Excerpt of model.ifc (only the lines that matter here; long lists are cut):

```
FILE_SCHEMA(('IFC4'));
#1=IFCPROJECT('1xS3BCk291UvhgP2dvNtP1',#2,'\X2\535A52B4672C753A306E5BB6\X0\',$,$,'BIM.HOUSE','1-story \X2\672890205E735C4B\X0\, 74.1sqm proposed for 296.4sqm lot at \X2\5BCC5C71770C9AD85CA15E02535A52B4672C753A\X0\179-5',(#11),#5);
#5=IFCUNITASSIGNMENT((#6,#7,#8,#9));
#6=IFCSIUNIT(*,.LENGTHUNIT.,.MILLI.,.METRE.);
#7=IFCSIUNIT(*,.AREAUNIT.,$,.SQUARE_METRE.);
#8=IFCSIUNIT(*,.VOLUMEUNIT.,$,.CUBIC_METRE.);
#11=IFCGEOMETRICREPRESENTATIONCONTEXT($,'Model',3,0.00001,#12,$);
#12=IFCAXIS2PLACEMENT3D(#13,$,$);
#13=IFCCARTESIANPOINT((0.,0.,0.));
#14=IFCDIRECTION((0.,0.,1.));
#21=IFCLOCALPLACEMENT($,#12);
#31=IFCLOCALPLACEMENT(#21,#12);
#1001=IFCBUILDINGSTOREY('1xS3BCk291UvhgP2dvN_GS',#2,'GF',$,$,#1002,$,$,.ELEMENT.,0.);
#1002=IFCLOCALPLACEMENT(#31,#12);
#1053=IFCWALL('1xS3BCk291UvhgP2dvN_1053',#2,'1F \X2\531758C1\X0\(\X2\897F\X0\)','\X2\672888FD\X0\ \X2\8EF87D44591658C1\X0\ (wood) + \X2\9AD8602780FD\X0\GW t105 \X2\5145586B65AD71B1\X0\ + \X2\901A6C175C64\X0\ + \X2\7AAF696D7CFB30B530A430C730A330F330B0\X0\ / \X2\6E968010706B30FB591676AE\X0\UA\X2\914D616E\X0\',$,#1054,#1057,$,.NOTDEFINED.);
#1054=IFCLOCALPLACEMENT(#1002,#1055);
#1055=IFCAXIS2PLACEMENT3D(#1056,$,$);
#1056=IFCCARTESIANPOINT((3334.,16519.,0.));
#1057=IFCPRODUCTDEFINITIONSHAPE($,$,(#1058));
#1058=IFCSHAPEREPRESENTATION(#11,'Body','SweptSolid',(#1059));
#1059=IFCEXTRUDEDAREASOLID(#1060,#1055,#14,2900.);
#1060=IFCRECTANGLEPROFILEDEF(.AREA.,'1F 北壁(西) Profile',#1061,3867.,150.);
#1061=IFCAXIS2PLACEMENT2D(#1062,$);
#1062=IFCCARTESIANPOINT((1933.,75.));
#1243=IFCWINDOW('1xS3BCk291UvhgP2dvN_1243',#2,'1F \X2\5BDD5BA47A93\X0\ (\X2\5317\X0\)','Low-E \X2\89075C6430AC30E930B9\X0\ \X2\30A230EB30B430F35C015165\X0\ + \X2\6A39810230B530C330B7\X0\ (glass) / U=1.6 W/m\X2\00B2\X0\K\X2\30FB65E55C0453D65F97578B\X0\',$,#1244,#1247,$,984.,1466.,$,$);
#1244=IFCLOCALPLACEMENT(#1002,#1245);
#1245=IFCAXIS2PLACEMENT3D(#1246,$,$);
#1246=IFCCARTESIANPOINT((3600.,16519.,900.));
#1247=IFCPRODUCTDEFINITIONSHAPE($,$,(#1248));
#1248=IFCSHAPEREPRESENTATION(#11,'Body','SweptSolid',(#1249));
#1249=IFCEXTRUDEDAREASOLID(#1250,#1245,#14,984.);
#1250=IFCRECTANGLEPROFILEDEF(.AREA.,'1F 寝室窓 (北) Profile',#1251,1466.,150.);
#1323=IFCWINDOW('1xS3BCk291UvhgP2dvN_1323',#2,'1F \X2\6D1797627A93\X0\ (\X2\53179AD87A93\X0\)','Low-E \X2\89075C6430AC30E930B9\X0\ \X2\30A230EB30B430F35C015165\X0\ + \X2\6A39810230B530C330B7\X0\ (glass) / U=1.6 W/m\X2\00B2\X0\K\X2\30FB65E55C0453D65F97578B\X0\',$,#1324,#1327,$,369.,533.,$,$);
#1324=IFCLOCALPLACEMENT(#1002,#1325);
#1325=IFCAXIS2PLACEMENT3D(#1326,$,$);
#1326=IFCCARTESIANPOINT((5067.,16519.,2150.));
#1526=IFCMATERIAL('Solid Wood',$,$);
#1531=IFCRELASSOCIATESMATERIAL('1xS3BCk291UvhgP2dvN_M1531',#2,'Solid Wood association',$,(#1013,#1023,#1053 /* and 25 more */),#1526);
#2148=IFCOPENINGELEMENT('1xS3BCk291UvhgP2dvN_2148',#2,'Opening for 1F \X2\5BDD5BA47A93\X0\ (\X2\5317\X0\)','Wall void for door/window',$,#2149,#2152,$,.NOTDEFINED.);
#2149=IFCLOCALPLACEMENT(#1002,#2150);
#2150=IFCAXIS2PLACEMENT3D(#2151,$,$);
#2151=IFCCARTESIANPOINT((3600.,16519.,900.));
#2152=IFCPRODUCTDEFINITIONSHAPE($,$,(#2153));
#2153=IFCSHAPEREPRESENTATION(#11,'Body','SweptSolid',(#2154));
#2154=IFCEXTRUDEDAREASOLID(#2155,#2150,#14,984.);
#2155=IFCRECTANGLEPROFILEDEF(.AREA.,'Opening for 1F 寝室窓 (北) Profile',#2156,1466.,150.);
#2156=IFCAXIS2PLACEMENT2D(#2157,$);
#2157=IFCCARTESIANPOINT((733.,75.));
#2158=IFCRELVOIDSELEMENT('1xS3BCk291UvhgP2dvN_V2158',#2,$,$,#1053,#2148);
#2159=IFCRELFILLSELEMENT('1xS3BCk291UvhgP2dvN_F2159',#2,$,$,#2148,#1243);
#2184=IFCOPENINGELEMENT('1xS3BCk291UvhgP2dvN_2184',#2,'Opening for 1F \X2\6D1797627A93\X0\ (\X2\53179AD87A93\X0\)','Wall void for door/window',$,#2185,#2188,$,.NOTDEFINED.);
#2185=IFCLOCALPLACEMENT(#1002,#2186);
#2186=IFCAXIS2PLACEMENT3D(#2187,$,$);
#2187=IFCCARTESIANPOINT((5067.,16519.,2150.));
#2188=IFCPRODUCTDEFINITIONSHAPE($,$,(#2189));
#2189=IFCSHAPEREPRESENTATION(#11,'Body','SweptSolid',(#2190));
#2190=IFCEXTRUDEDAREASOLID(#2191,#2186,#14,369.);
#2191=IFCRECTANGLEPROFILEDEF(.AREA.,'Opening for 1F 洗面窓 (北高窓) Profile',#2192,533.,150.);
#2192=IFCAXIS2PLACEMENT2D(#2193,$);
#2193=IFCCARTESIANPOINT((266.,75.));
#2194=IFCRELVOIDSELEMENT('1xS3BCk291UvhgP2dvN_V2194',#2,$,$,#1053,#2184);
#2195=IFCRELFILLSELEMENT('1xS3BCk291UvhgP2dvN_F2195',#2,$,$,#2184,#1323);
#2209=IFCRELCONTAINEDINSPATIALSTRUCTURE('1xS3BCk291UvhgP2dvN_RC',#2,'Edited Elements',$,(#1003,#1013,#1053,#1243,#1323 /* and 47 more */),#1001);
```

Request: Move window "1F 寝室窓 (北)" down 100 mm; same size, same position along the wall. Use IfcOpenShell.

```python
import numpy as np
import ifcopenshell
import ifcopenshell.api.geometry
import ifcopenshell.util.placement
import ifcopenshell.util.unit

model = ifcopenshell.open("model.ifc")
unit_scale = ifcopenshell.util.unit.calculate_unit_scale(model)

window = model.by_guid("1xS3BCk291UvhgP2dvN_1243")
opening = window.FillsVoids[0].RelatingOpeningElement
dz = -0.1 / unit_scale

shift = np.array([0.0, 0.0, dz])
# The window is not placed relative to its opening, so move both.
for product in (opening, window):
    matrix = ifcopenshell.util.placement.get_local_placement(product.ObjectPlacement)
    matrix[:3, 3] += shift
    ifcopenshell.api.geometry.edit_object_placement(model, product=product, matrix=matrix, is_si=False)

print(f"moved by {dz * unit_scale:+.3f} m")

model.write("model_updated.ifc")
```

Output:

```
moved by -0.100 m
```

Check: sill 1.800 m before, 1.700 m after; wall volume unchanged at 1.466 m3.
